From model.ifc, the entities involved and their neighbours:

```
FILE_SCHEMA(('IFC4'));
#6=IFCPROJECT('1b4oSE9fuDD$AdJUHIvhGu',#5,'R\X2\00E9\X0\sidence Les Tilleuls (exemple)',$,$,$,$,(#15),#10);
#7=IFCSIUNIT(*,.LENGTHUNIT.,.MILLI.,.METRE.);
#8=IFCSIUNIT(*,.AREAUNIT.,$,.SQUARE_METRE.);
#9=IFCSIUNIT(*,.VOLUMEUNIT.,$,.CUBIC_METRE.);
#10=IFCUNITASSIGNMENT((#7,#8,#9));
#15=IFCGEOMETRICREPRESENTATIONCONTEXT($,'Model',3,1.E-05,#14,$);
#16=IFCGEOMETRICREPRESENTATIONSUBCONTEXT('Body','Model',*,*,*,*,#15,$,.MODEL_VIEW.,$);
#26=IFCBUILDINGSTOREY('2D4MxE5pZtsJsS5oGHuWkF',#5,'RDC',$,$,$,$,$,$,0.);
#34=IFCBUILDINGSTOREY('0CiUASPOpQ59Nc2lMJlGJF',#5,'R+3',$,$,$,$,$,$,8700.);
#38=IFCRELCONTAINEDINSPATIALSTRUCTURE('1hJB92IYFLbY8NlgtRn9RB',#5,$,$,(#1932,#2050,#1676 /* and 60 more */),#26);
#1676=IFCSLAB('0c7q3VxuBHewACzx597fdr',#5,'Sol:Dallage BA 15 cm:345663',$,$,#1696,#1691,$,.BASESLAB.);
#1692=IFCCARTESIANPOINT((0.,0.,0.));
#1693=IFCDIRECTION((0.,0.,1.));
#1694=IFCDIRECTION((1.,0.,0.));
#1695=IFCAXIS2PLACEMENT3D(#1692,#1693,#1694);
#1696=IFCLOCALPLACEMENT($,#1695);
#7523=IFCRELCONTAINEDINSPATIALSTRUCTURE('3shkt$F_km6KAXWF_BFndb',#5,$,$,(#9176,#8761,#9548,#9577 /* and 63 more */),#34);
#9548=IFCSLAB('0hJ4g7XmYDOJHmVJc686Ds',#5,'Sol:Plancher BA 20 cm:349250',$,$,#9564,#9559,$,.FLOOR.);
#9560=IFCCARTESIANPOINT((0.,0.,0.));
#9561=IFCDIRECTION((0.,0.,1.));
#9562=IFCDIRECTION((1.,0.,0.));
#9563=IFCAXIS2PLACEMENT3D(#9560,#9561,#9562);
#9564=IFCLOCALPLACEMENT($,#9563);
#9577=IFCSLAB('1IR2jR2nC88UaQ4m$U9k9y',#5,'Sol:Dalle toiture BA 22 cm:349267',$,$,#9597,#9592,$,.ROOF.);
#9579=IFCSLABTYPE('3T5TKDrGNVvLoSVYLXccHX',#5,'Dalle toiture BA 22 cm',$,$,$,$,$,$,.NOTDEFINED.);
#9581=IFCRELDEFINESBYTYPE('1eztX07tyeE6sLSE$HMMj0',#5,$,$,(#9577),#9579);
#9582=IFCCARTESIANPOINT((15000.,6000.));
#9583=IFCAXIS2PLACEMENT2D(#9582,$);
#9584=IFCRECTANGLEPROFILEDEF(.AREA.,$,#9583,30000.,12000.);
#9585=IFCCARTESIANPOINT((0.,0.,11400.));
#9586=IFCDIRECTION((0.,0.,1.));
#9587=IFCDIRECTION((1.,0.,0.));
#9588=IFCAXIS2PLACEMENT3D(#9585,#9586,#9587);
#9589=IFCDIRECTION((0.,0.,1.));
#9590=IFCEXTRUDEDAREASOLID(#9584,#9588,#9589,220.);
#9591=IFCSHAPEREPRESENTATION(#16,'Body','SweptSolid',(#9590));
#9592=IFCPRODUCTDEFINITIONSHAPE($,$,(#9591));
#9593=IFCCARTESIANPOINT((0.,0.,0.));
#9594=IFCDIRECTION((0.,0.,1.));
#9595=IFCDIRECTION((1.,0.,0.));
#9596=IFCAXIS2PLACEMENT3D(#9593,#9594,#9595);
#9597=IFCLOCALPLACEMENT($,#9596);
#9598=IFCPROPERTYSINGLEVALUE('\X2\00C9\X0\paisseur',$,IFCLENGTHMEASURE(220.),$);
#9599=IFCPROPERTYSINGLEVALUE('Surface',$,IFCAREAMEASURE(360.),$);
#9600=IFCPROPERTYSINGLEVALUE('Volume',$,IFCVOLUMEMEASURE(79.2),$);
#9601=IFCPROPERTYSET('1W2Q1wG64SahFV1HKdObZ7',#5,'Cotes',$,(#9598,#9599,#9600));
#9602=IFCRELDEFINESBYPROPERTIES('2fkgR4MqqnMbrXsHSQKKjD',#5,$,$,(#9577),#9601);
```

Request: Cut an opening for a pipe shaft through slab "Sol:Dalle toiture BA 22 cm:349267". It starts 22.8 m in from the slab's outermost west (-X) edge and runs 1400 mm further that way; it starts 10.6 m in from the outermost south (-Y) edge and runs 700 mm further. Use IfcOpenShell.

```python
import numpy as np
import ifcopenshell
import ifcopenshell.api.feature
import ifcopenshell.api.geometry
import ifcopenshell.api.pset
import ifcopenshell.api.root
import ifcopenshell.geom
import ifcopenshell.util.element
import ifcopenshell.util.placement
import ifcopenshell.util.representation
import ifcopenshell.util.shape
import ifcopenshell.util.unit

model = ifcopenshell.open("model.ifc")
unit_scale = ifcopenshell.util.unit.calculate_unit_scale(model)
area_scale = ifcopenshell.util.unit.calculate_unit_scale(model, "AREAUNIT")
volume_scale = ifcopenshell.util.unit.calculate_unit_scale(model, "VOLUMEUNIT")
settings = ifcopenshell.geom.settings()


def volume(element):
    """Net volume in cubic metres, openings subtracted."""
    shape = ifcopenshell.geom.create_shape(settings, element)
    return ifcopenshell.util.shape.get_volume(shape.geometry)


slab = model.by_guid("1IR2jR2nC88UaQ4m$U9k9y")
before = volume(slab)

# Extent in the slab's own axes, in metres. The edges named are its -X and -Y sides.
slab_shape = ifcopenshell.geom.create_shape(settings, slab)
vertices = ifcopenshell.util.shape.get_vertices(slab_shape.geometry)
x_min, y_min, bottom = vertices.min(axis=0)
top = vertices[:, 2].max()

opening = ifcopenshell.api.root.create_entity(model, ifc_class="IfcOpeningElement", name="Pipe shaft opening", predefined_type="OPENING")
context = ifcopenshell.util.representation.get_context(model, "Model", "Body", "MODEL_VIEW")
width, depth = 1.4, 0.7
outline = [(0.0, 0.0), (width, 0.0), (width, depth), (0.0, depth), (0.0, 0.0)]
# Overshoot both faces by 50 mm so the cut is clean.
shape = ifcopenshell.api.geometry.add_slab_representation(
    model, context=context, depth=top - bottom + 0.1, polyline=outline
)
ifcopenshell.api.geometry.assign_representation(model, product=opening, representation=shape)

matrix = ifcopenshell.util.placement.get_local_placement(slab.ObjectPlacement)
matrix[:, 3] = matrix @ np.append(np.array([x_min + 22.8, y_min + 10.6, bottom - 0.05]) / unit_scale, 1.0)
ifcopenshell.api.geometry.edit_object_placement(model, product=opening, matrix=matrix, is_si=False)
ifcopenshell.api.feature.add_feature(model, feature=opening, element=slab)

after = volume(slab)

# Update the slab's stored quantities.
pset = model.by_id(ifcopenshell.util.element.get_pset(slab, "Cotes", should_inherit=False)["id"])
ifcopenshell.api.pset.edit_pset(model, pset=pset, properties={
    "Surface": model.create_entity("IfcAreaMeasure", after / (top - bottom) / area_scale),
    "Volume": model.create_entity("IfcVolumeMeasure", after / volume_scale),
})

print(f"slab volume {before:.3f} -> {after:.3f} m3")

model.write("model_updated.ifc")
```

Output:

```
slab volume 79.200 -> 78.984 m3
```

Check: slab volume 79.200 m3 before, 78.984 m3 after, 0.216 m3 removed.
